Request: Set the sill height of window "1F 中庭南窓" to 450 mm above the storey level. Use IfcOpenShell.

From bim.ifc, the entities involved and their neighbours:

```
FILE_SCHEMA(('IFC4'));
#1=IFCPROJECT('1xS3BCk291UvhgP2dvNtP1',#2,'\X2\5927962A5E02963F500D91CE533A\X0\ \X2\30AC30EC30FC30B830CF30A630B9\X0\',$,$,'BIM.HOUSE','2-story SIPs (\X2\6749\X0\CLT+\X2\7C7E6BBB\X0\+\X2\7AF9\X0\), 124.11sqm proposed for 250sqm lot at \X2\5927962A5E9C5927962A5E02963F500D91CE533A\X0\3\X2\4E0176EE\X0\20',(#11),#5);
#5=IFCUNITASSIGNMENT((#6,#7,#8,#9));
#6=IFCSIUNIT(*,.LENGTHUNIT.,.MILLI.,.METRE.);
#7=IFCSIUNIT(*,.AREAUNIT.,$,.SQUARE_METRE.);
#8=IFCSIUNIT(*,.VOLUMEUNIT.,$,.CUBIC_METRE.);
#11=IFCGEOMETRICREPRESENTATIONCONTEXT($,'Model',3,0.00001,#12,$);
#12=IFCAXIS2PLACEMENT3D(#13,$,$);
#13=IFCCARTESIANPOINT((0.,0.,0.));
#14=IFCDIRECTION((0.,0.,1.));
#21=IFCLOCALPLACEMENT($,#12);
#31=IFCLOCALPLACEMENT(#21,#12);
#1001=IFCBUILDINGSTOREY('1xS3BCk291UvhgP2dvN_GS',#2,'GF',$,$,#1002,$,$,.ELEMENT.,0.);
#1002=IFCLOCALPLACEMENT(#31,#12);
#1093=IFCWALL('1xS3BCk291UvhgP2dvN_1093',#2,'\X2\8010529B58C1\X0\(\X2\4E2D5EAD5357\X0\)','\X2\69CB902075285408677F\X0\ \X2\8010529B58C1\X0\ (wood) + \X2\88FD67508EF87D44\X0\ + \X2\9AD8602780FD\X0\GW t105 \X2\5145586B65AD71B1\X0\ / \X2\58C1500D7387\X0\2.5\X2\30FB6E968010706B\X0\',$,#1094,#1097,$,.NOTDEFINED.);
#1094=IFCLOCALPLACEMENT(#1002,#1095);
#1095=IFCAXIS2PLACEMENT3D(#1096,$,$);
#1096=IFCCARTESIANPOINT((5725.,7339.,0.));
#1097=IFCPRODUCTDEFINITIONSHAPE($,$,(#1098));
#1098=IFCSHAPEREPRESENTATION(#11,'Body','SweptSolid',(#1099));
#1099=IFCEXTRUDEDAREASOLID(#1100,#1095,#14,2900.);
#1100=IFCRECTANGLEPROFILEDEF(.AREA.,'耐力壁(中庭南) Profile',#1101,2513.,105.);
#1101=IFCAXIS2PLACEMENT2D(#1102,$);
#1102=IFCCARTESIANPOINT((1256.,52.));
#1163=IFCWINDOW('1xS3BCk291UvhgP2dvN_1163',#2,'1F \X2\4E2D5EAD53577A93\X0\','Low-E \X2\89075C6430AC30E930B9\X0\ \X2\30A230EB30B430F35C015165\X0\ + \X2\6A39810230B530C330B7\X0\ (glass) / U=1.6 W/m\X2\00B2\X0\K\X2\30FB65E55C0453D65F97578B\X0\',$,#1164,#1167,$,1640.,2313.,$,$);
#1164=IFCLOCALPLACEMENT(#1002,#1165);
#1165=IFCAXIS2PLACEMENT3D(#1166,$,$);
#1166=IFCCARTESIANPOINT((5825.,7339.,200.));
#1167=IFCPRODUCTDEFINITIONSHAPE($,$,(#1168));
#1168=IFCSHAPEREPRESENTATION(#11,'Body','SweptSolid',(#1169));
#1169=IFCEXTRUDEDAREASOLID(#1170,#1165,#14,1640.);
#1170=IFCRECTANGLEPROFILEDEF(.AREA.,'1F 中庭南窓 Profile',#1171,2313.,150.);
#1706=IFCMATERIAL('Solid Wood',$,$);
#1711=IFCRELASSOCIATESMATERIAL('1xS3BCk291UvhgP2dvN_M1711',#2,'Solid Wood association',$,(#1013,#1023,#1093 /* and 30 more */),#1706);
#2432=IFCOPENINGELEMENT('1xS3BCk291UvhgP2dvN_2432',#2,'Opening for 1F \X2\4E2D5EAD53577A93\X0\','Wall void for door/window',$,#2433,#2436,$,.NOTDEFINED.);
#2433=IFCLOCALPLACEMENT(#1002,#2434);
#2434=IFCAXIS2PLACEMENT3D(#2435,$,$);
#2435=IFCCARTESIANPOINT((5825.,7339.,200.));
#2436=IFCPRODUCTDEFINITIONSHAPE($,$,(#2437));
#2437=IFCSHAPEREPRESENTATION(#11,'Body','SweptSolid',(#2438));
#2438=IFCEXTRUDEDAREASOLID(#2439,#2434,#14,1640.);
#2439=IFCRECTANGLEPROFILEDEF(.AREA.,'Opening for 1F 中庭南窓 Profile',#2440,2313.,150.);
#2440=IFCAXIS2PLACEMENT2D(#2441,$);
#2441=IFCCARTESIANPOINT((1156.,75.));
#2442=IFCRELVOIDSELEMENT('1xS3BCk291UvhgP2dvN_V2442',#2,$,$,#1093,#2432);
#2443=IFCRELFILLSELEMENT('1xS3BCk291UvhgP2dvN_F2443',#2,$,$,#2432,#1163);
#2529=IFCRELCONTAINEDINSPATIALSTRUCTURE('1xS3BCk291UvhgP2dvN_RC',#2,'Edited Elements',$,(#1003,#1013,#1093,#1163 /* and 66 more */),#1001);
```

```python
import numpy as np
import ifcopenshell
import ifcopenshell.api.geometry
import ifcopenshell.geom
import ifcopenshell.util.element
import ifcopenshell.util.placement
import ifcopenshell.util.shape
import ifcopenshell.util.unit

model = ifcopenshell.open("bim.ifc")
unit_scale = ifcopenshell.util.unit.calculate_unit_scale(model)

window = model.by_guid("1xS3BCk291UvhgP2dvN_1163")
opening = window.FillsVoids[0].RelatingOpeningElement
storey = ifcopenshell.util.element.get_container(window, ifc_class="IfcBuildingStorey")
level = ifcopenshell.util.placement.get_local_placement(storey.ObjectPlacement)[2, 3]

# The opening's origin need not be at the sill, so measure its lowest point.
shape = ifcopenshell.geom.create_shape(ifcopenshell.geom.settings(), opening)
bottom = ifcopenshell.util.shape.get_shape_bottom_elevation(shape, shape.geometry) / unit_scale
dz = level + 450.0 - bottom

shift = np.array([0.0, 0.0, dz])
# The window is not placed relative to its opening, so move both.
for product in (opening, window):
    matrix = ifcopenshell.util.placement.get_local_placement(product.ObjectPlacement)
    matrix[:3, 3] += shift
    ifcopenshell.api.geometry.edit_object_placement(model, product=product, matrix=matrix, is_si=False)

print(f"moved by {dz * unit_scale:+.3f} m")

model.write("bim_rev.ifc")
```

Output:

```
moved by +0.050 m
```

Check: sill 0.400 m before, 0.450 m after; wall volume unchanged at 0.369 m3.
